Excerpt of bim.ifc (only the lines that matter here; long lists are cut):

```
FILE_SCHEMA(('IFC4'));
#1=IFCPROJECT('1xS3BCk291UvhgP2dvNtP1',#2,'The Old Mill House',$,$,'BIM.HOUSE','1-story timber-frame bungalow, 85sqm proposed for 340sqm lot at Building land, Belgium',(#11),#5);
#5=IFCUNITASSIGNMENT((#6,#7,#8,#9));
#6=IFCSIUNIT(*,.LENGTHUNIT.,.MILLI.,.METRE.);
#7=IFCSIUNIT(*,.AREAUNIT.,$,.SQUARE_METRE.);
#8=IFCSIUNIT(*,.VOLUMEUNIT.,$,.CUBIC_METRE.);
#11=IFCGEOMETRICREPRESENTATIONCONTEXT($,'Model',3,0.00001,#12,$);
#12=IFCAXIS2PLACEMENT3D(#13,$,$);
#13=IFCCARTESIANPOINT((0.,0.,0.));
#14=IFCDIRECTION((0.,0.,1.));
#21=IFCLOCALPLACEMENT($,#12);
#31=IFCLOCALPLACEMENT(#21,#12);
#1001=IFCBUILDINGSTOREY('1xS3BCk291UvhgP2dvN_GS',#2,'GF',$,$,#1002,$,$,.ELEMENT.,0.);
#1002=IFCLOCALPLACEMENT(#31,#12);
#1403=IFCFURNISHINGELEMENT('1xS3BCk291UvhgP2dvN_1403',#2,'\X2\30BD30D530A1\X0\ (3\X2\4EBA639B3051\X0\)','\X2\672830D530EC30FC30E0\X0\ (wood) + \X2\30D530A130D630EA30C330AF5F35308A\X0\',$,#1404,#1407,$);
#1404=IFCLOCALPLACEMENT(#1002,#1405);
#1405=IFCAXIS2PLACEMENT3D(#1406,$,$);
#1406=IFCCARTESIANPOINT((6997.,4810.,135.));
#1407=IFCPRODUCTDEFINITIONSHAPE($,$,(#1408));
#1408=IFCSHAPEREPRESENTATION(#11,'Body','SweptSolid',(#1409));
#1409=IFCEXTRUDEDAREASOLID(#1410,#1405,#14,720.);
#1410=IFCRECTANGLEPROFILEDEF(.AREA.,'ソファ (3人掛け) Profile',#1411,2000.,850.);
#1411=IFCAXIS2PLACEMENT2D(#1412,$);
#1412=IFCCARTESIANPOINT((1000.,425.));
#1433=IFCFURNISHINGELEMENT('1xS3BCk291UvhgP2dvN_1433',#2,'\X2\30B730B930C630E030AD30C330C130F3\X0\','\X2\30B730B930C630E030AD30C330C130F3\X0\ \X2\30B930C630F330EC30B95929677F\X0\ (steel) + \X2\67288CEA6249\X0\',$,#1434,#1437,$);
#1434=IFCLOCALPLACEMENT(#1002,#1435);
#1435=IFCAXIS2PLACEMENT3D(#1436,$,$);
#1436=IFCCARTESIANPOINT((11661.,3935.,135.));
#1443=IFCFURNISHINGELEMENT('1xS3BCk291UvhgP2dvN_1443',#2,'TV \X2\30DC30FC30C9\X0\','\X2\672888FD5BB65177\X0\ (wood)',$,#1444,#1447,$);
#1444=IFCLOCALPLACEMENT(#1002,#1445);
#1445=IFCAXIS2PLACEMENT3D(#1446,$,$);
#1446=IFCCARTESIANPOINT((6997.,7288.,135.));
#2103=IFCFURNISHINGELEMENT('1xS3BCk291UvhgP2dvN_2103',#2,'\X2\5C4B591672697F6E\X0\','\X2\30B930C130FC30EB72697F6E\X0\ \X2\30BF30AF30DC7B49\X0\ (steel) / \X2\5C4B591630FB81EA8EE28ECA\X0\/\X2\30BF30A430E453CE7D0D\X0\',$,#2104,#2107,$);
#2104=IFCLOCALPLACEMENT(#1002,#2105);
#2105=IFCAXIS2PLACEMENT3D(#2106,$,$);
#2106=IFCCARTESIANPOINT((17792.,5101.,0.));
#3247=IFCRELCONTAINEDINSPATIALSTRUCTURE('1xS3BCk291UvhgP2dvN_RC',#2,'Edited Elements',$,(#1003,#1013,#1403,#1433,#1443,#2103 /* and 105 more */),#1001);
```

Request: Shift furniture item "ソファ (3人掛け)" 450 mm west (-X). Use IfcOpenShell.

```python
import ifcopenshell
import ifcopenshell.api.geometry
import ifcopenshell.util.placement

model = ifcopenshell.open("bim.ifc")

item = model.by_guid("1xS3BCk291UvhgP2dvN_1403")
matrix = ifcopenshell.util.placement.get_local_placement(item.ObjectPlacement)
matrix[0, 3] -= 450.0
ifcopenshell.api.geometry.edit_object_placement(model, product=item, matrix=matrix, is_si=False)

print(ifcopenshell.util.placement.get_local_placement(item.ObjectPlacement).round(3) + 0.0)

model.write("bim-out.ifc")
```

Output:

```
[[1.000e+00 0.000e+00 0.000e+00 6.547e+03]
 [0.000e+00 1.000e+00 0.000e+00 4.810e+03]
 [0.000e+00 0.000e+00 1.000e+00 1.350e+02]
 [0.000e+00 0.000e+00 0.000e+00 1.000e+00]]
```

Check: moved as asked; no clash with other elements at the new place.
